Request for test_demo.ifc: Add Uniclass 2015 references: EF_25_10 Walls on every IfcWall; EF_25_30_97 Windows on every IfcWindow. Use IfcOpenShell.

First a look at what the model holds.

```python
import ifcopenshell

model = ifcopenshell.open("test_demo.ifc")
print(model.schema)
print("classifications:", [c.Name for c in model.by_type("IfcClassification")])
for ifc_class in ("IfcDoor", "IfcRoof", "IfcStair", "IfcWall", "IfcWindow"):
    print(ifc_class, len(model.by_type(ifc_class)))
```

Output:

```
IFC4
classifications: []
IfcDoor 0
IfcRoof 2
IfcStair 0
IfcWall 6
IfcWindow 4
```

```python
import ifcopenshell
import ifcopenshell.api.classification

model = ifcopenshell.open("test_demo.ifc")

system = ifcopenshell.api.classification.add_classification(model, classification="Uniclass 2015")

codes = {
    "IfcWall": ("EF_25_10", "Walls"),
    "IfcWindow": ("EF_25_30_97", "Windows"),
}
for ifc_class, (code, name) in codes.items():
    products = model.by_type(ifc_class)
    ifcopenshell.api.classification.add_reference(
        model, products=products, classification=system, identification=code, name=name
    )
    print(code, len(products))

model.write("test_demo_rev.ifc")
```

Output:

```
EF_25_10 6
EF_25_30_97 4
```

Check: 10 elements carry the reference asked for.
